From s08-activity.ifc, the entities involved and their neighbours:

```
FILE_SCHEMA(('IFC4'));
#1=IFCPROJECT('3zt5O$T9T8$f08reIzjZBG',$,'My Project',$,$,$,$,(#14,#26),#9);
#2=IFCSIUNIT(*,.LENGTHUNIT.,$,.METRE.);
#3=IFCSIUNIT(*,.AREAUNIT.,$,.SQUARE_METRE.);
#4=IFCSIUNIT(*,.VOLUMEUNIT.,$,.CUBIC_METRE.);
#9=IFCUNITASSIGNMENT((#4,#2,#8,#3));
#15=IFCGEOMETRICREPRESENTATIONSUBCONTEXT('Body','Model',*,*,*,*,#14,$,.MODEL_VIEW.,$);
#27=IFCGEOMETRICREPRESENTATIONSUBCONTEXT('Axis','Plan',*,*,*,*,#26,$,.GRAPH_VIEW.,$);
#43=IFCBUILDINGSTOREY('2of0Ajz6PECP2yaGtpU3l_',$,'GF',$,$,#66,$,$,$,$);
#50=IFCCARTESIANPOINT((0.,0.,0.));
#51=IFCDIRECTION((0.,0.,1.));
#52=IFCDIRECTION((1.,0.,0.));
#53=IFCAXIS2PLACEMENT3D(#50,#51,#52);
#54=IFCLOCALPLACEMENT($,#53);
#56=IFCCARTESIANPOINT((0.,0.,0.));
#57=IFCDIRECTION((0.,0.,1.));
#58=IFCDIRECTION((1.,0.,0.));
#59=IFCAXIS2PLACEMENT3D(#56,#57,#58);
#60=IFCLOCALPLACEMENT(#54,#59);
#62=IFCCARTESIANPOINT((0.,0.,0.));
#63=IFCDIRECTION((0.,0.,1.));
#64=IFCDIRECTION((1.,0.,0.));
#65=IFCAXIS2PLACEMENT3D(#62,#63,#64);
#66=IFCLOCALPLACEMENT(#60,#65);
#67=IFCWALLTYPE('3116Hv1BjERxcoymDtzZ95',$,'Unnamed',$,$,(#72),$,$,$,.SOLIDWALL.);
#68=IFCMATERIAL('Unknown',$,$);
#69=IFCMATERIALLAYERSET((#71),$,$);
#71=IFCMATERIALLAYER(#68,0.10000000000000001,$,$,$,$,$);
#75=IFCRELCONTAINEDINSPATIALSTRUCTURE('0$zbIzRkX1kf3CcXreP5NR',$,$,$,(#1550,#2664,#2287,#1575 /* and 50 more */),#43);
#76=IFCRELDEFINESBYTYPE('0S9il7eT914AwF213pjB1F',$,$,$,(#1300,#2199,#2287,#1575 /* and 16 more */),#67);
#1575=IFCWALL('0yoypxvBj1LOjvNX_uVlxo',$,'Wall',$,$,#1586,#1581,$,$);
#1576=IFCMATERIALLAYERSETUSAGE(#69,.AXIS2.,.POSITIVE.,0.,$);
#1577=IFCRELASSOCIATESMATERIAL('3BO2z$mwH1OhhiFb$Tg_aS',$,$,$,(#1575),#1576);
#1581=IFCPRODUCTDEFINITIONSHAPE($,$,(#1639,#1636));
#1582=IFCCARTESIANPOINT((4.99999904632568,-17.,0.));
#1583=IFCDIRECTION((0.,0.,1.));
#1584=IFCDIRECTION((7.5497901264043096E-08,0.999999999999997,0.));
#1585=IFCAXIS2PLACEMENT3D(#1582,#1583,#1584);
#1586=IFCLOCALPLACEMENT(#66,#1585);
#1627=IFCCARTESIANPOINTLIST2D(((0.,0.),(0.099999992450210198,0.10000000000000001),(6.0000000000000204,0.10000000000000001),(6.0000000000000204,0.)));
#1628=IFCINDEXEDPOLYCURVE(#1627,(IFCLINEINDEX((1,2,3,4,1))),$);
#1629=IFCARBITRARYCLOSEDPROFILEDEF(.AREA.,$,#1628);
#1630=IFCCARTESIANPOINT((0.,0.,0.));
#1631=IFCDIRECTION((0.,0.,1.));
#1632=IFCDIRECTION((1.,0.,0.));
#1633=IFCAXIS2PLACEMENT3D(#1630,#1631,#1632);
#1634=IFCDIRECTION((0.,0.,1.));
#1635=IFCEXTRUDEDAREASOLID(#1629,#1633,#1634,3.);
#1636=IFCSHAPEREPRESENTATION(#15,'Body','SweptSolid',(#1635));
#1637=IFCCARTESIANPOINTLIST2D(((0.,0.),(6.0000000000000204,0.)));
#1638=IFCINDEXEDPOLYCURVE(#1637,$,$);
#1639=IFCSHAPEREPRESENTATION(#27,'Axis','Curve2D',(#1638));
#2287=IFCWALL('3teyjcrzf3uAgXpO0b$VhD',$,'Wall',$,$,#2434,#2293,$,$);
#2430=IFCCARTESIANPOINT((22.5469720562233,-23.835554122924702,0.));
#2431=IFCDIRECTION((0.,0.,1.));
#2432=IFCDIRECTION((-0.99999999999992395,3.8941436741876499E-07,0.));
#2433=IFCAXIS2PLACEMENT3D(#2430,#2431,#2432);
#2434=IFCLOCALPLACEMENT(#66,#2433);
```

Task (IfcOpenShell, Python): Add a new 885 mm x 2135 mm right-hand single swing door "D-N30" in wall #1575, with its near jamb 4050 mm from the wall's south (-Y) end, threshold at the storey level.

```python
import numpy as np
import ifcopenshell
import ifcopenshell.api.feature
import ifcopenshell.api.geometry
import ifcopenshell.api.root
import ifcopenshell.api.spatial
import ifcopenshell.geom
import ifcopenshell.util.element
import ifcopenshell.util.placement
import ifcopenshell.util.representation
import ifcopenshell.util.shape
import ifcopenshell.util.unit

model = ifcopenshell.open("s08-activity.ifc")
unit_scale = ifcopenshell.util.unit.calculate_unit_scale(model)
settings = ifcopenshell.geom.settings()


def volume(element):
    """Net volume in cubic metres, openings subtracted."""
    shape = ifcopenshell.geom.create_shape(settings, element)
    return ifcopenshell.util.shape.get_volume(shape.geometry)


wall = model.by_guid("0yoypxvBj1LOjvNX_uVlxo")
storey = ifcopenshell.util.element.get_container(wall, ifc_class="IfcBuildingStorey")
context = ifcopenshell.util.representation.get_context(model, "Model", "Body", "MODEL_VIEW")
before = volume(wall)

width, height, from_end, sill = 0.885, 2.135, 4.05, 0.0  # metres

# The wall runs along its own X axis, and the end named is its -X end.
wall_shape = ifcopenshell.geom.create_shape(settings, wall)
x, y, z = ifcopenshell.util.shape.get_vertices(wall_shape.geometry).T
start = x.min() + from_end
face, thickness = float(y.min()), float(y.max() - y.min())
wall_matrix = ifcopenshell.util.placement.get_local_placement(wall.ObjectPlacement)
level = ifcopenshell.util.placement.get_local_placement(storey.ObjectPlacement)[2, 3]


def in_wall(x, y):
    """Placement at x, y metres in the wall's axes, at sill height."""
    matrix = wall_matrix.copy()
    matrix[:, 3] = wall_matrix @ np.array([x / unit_scale, y / unit_scale, 0.0, 1.0])
    matrix[2, 3] = level + sill / unit_scale
    return matrix


# Opening: a box that overshoots both wall faces by 50 mm.
opening = ifcopenshell.api.root.create_entity(model, ifc_class="IfcOpeningElement", predefined_type="OPENING")
box = ifcopenshell.api.geometry.add_wall_representation(
    model, context=context, length=width, height=height, thickness=thickness + 0.1
)
ifcopenshell.api.geometry.assign_representation(model, product=opening, representation=box)
ifcopenshell.api.geometry.edit_object_placement(model, product=opening, matrix=in_wall(start, face - 0.05), is_si=False)
ifcopenshell.api.feature.add_feature(model, feature=opening, element=wall)

door = ifcopenshell.api.root.create_entity(model, ifc_class="IfcDoor", name="D-N30", predefined_type="DOOR")
door.OverallWidth, door.OverallHeight = width / unit_scale, height / unit_scale
door.OperationType = "SINGLE_SWING_RIGHT"
body = ifcopenshell.api.geometry.add_door_representation(
    model,
    context=context,
    overall_width=door.OverallWidth,
    overall_height=door.OverallHeight,
    operation_type="SINGLE_SWING_RIGHT",
    lining_properties={"LiningDepth": thickness / unit_scale, "ThresholdDepth": thickness / unit_scale},
)
ifcopenshell.api.geometry.assign_representation(model, product=door, representation=body)
ifcopenshell.api.spatial.assign_container(model, products=[door], relating_structure=storey)
ifcopenshell.api.feature.add_filling(model, opening=opening, element=door)

# The lining spans the wall, so the door starts at the wall face.
ifcopenshell.api.geometry.edit_object_placement(model, product=door, matrix=in_wall(start, face), is_si=False)

after = volume(wall)

print(f"wall volume {before:.3f} -> {after:.3f} m3")

model.write("s08-activity-out.ifc")
```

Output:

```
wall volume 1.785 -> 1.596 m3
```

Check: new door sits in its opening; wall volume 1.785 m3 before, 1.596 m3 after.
